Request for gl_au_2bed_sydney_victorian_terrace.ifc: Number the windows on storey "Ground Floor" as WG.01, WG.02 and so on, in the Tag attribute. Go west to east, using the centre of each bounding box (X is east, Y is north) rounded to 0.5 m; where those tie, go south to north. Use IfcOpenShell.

First a look at what the model holds.

```python
import ifcopenshell
import ifcopenshell.util.element
import ifcopenshell.util.placement

model = ifcopenshell.open("gl_au_2bed_sydney_victorian_terrace.ifc")
print(model.schema)
storey = next(s for s in model.by_type("IfcBuildingStorey") if s.Name == "Ground Floor")
windows = [e for e in ifcopenshell.util.element.get_decomposition(storey) if e.is_a("IfcWindow")]
for e in sorted(windows, key=lambda e: e.id()):
    origin = ifcopenshell.util.placement.get_local_placement(e.ObjectPlacement)[:3, 3]
    print(e.id(), e.Tag, e.Name, origin.round(2) + 0.0, sep=" | ")
```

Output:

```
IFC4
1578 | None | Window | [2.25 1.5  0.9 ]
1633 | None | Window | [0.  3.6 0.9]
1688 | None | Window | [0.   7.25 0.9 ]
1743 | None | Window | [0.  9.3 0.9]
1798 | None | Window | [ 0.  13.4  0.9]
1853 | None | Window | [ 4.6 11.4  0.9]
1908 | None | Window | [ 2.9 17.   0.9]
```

```python
import ifcopenshell
import ifcopenshell.geom
import ifcopenshell.util.element
import ifcopenshell.util.shape

model = ifcopenshell.open("gl_au_2bed_sydney_victorian_terrace.ifc")
settings = ifcopenshell.geom.settings()
settings.set("use-world-coords", True)


def centre(element):
    shape = ifcopenshell.geom.create_shape(settings, element)
    return ifcopenshell.util.shape.get_bbox_centroid(shape.geometry)


storey = next(s for s in model.by_type("IfcBuildingStorey") if s.Name == "Ground Floor")
windows = [e for e in ifcopenshell.util.element.get_decomposition(storey) if e.is_a("IfcWindow")]

# Insertion points can sit at a corner or the storey origin, so sort by the geometry (in metres).
centres = {e: centre(e) for e in windows}
windows.sort(key=lambda e: (round(centres[e][0] / 0.5), centres[e][1]))

for i, e in enumerate(windows, start=1):
    number = f"WG.{i:02d}"
    e.Tag = number
    print(e.id(), number)

model.write("gl_au_2bed_sydney_victorian_terrace_rev.ifc")
```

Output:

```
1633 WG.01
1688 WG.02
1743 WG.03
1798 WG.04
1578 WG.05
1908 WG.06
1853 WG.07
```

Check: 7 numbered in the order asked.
